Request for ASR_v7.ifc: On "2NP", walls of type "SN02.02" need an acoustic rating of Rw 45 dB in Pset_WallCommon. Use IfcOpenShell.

First a look at what the model holds.

```python
import ifcopenshell
import ifcopenshell.util.element

model = ifcopenshell.open("ASR_v7.ifc")
print(model.schema)
storey = next(s for s in model.by_type("IfcBuildingStorey") if s.Name == "2NP")
walls = [e for e in ifcopenshell.util.element.get_decomposition(storey) if e.is_a("IfcWall")]
seen = {}
for e in walls:
    element_type = ifcopenshell.util.element.get_type(e)
    key = (element_type.Name if element_type != e and element_type else None, ifcopenshell.util.element.get_pset(e, "Pset_WallCommon", "AcousticRating"))
    seen[key] = seen.get(key, 0) + 1
for (name, value), count in sorted(seen.items(), key=str):
    print(count, "x", name, "|", value)
```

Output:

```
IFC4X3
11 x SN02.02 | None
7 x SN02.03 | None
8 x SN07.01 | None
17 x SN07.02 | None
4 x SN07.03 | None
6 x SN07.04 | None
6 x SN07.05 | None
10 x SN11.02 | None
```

```python
import ifcopenshell
import ifcopenshell.api.pset
import ifcopenshell.util.element

model = ifcopenshell.open("ASR_v7.ifc")

storey = next(s for s in model.by_type("IfcBuildingStorey") if s.Name == "2NP")
walls = [e for e in ifcopenshell.util.element.get_decomposition(storey) if e.is_a("IfcWall")]

count = 0
for e in walls:
    element_type = ifcopenshell.util.element.get_type(e)
    if element_type in (None, e) or element_type.Name != "SN02.02":
        continue
    # add_pset returns the element's existing set when there is one.
    pset = ifcopenshell.api.pset.add_pset(model, product=e, name="Pset_WallCommon")
    ifcopenshell.api.pset.edit_pset(model, pset=pset, properties={"AcousticRating": "Rw 45 dB"})
    count += 1

print(count, "walls updated")

model.write("ASR_v7_edited.ifc")
```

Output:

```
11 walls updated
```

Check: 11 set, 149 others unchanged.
